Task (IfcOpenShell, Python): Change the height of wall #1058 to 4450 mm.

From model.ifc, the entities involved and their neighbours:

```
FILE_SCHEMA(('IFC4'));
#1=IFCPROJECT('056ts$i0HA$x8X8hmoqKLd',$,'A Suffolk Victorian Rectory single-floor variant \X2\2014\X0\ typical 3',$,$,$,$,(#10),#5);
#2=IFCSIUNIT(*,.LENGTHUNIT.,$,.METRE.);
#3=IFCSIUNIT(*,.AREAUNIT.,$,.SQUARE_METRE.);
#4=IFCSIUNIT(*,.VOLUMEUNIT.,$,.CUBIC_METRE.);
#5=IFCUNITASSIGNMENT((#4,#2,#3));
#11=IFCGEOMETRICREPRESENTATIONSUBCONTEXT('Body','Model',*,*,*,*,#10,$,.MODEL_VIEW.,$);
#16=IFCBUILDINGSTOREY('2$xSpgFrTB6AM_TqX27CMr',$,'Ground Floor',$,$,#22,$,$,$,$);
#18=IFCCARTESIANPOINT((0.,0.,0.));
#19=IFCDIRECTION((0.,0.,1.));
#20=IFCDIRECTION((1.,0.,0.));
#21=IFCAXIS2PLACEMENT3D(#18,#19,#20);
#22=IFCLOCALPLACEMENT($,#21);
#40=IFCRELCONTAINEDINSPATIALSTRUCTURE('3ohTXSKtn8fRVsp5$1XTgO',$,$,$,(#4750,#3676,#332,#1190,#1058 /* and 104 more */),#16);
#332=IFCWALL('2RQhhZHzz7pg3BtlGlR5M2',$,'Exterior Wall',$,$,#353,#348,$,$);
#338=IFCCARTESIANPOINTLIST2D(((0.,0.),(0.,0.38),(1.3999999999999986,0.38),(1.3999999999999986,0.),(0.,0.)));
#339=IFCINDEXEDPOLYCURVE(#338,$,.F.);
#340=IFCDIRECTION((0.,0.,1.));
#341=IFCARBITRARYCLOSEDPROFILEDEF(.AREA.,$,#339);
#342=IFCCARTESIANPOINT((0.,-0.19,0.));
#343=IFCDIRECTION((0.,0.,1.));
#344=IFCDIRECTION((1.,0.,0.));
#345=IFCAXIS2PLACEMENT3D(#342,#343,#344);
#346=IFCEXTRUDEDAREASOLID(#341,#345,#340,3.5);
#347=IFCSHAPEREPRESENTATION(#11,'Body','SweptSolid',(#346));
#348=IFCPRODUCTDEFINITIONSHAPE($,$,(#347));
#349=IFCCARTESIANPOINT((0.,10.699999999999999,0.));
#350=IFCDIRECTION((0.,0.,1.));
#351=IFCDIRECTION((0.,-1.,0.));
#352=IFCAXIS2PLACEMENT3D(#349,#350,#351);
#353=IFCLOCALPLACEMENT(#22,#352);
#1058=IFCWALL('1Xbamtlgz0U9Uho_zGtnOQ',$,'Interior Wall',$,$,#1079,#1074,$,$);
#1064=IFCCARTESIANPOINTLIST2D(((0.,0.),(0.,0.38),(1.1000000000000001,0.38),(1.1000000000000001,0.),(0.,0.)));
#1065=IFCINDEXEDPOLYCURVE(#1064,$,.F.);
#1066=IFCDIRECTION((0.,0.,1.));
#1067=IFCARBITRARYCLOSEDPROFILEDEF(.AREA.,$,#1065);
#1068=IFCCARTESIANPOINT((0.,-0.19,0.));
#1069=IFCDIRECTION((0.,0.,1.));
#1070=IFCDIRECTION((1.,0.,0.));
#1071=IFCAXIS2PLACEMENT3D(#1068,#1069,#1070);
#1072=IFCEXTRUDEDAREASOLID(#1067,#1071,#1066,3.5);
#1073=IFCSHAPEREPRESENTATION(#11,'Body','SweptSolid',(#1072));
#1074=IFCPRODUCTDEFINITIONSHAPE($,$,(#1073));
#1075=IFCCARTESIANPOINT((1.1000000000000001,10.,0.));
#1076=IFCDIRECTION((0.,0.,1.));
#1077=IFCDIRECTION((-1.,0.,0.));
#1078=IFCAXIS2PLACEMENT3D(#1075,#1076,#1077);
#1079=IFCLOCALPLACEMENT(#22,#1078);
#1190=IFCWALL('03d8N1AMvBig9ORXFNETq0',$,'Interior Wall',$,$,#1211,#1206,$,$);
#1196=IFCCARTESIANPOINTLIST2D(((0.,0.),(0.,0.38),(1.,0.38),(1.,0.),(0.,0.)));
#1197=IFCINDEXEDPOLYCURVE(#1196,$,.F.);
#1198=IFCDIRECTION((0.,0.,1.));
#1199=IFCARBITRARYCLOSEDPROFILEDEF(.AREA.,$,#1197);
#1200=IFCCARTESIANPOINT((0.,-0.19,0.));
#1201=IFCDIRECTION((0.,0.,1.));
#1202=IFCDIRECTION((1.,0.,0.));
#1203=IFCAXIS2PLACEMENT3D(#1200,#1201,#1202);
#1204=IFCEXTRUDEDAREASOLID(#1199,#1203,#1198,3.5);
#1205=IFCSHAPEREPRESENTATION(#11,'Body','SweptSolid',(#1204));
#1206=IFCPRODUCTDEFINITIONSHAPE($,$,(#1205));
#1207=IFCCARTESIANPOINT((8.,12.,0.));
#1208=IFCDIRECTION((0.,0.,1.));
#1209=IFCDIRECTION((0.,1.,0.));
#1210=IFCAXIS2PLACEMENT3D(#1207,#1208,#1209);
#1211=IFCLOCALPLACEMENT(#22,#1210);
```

```python
import ifcopenshell
import ifcopenshell.geom
import ifcopenshell.util.representation
import ifcopenshell.util.shape

model = ifcopenshell.open("model.ifc")
settings = ifcopenshell.geom.settings()


def volume(element):
    """Net volume in cubic metres, openings subtracted."""
    shape = ifcopenshell.geom.create_shape(settings, element)
    return ifcopenshell.util.shape.get_volume(shape.geometry)


wall = model.by_guid("1Xbamtlgz0U9Uho_zGtnOQ")
before = volume(wall)

body = ifcopenshell.util.representation.get_representation(wall, "Model", "Body")
solid = body.Items[0]
old_height = solid.Depth
solid.Depth = 4.45
after = volume(wall)

print(f"height {old_height:g} -> {solid.Depth:g}, volume {before:.3f} -> {after:.3f} m3")

model.write("model_v2.ifc")
```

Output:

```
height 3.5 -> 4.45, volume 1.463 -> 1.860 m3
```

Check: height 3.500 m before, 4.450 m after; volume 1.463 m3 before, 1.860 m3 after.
